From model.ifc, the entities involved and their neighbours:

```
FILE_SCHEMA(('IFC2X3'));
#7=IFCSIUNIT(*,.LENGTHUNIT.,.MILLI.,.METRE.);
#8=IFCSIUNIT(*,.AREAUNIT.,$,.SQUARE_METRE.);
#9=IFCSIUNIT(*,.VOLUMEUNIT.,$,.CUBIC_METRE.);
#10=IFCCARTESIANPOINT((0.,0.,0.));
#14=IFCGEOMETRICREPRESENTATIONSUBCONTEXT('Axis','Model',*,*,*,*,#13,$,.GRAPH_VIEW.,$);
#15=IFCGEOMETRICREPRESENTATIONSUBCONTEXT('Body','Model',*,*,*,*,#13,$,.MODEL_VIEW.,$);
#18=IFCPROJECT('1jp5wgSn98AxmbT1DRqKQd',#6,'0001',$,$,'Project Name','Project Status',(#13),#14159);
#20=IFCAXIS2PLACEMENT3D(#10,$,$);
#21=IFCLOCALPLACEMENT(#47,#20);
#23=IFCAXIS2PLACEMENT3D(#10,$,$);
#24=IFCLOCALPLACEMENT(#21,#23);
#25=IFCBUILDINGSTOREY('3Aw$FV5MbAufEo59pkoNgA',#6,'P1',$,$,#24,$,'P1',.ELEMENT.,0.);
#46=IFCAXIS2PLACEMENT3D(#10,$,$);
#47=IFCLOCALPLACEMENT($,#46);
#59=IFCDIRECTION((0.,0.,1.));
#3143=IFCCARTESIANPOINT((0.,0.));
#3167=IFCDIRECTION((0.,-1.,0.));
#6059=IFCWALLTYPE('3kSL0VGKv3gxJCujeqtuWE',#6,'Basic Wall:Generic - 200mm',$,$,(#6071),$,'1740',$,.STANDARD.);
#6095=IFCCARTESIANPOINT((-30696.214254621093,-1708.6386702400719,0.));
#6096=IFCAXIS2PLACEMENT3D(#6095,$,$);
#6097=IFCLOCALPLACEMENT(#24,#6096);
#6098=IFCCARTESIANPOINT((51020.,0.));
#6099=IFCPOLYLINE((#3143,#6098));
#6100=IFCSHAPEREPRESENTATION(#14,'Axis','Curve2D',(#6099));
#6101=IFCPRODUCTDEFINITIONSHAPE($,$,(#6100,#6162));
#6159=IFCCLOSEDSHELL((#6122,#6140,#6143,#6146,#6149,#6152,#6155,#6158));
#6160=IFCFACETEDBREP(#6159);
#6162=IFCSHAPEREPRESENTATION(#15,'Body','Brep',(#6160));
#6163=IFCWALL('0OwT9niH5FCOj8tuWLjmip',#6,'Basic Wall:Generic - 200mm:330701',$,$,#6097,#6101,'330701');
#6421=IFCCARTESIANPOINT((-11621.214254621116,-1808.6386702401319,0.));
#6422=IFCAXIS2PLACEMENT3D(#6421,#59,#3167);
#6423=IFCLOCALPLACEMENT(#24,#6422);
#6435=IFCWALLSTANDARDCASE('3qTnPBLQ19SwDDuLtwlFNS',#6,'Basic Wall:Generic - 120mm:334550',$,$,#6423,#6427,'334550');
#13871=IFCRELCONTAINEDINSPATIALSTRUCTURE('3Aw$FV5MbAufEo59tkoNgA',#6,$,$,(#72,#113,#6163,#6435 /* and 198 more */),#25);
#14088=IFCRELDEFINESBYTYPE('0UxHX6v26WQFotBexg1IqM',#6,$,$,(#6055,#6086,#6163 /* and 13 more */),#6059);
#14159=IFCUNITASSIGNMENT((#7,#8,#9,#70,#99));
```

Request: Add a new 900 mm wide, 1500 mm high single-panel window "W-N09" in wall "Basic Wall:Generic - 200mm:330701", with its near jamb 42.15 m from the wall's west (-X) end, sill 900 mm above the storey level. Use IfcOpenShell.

```python
import numpy as np
import ifcopenshell
import ifcopenshell.api.feature
import ifcopenshell.api.geometry
import ifcopenshell.api.root
import ifcopenshell.api.spatial
import ifcopenshell.api.type
import ifcopenshell.geom
import ifcopenshell.util.element
import ifcopenshell.util.placement
import ifcopenshell.util.representation
import ifcopenshell.util.shape
import ifcopenshell.util.unit

model = ifcopenshell.open("model.ifc")
unit_scale = ifcopenshell.util.unit.calculate_unit_scale(model)
settings = ifcopenshell.geom.settings()


def volume(element):
    """Net volume in cubic metres, openings subtracted."""
    shape = ifcopenshell.geom.create_shape(settings, element)
    return ifcopenshell.util.shape.get_volume(shape.geometry)


wall = model.by_guid("0OwT9niH5FCOj8tuWLjmip")
storey = ifcopenshell.util.element.get_container(wall, ifc_class="IfcBuildingStorey")
context = ifcopenshell.util.representation.get_context(model, "Model", "Body", "MODEL_VIEW")
before = volume(wall)

width, height, from_end, sill = 0.9, 1.5, 42.15, 0.9  # metres

# The wall runs along its own X axis, and the end named is its -X end.
wall_shape = ifcopenshell.geom.create_shape(settings, wall)
x, y, z = ifcopenshell.util.shape.get_vertices(wall_shape.geometry).T
start = x.min() + from_end
face, thickness = float(y.min()), float(y.max() - y.min())
wall_matrix = ifcopenshell.util.placement.get_local_placement(wall.ObjectPlacement)
level = ifcopenshell.util.placement.get_local_placement(storey.ObjectPlacement)[2, 3]


def in_wall(x, y):
    """Placement at x, y metres in the wall's axes, at sill height."""
    matrix = wall_matrix.copy()
    matrix[:, 3] = wall_matrix @ np.array([x / unit_scale, y / unit_scale, 0.0, 1.0])
    matrix[2, 3] = level + sill / unit_scale
    return matrix


# Opening: a box that overshoots both wall faces by 50 mm.
opening = ifcopenshell.api.root.create_entity(model, ifc_class="IfcOpeningElement")
box = ifcopenshell.api.geometry.add_wall_representation(
    model, context=context, length=width, height=height, thickness=thickness + 0.1
)
ifcopenshell.api.geometry.assign_representation(model, product=opening, representation=box)
ifcopenshell.api.geometry.edit_object_placement(model, product=opening, matrix=in_wall(start, face - 0.05), is_si=False)
ifcopenshell.api.feature.add_feature(model, feature=opening, element=wall)

window = ifcopenshell.api.root.create_entity(model, ifc_class="IfcWindow", name="W-N09")
window.OverallWidth, window.OverallHeight = width / unit_scale, height / unit_scale
body = ifcopenshell.api.geometry.add_window_representation(
    model,
    context=context,
    overall_width=window.OverallWidth,
    overall_height=window.OverallHeight,
    partition_type="SINGLE_PANEL",
)
ifcopenshell.api.geometry.assign_representation(model, product=window, representation=body)
ifcopenshell.api.spatial.assign_container(model, products=[window], relating_structure=storey)
fills = ifcopenshell.api.feature.add_filling(model, opening=opening, element=window)
fills.OwnerHistory = window.OwnerHistory  # required in IFC2X3

# IFC2X3 keeps the operation on the window style.
style = ifcopenshell.api.root.create_entity(model, ifc_class="IfcWindowStyle", name="W-N09")
style.OperationType, style.ConstructionType = "SINGLE_PANEL", "NOTDEFINED"
style.ParameterTakesPrecedence = style.Sizeable = False
ifcopenshell.api.type.assign_type(model, related_objects=[window], relating_type=style)

# Centre the window in the wall's thickness.
ifcopenshell.api.geometry.edit_object_placement(model, product=window, matrix=in_wall(start, face), is_si=False)
window_shape = ifcopenshell.geom.create_shape(settings, window)
depth = ifcopenshell.util.shape.get_vertices(window_shape.geometry)[:, 1]
offset = face + thickness / 2 - (depth.min() + depth.max()) / 2
ifcopenshell.api.geometry.edit_object_placement(model, product=window, matrix=in_wall(start, offset), is_si=False)

after = volume(wall)

print(f"wall volume {before:.3f} -> {after:.3f} m3")

model.write("model_updated.ifc")
```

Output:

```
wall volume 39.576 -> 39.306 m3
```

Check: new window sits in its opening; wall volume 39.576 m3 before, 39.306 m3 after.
